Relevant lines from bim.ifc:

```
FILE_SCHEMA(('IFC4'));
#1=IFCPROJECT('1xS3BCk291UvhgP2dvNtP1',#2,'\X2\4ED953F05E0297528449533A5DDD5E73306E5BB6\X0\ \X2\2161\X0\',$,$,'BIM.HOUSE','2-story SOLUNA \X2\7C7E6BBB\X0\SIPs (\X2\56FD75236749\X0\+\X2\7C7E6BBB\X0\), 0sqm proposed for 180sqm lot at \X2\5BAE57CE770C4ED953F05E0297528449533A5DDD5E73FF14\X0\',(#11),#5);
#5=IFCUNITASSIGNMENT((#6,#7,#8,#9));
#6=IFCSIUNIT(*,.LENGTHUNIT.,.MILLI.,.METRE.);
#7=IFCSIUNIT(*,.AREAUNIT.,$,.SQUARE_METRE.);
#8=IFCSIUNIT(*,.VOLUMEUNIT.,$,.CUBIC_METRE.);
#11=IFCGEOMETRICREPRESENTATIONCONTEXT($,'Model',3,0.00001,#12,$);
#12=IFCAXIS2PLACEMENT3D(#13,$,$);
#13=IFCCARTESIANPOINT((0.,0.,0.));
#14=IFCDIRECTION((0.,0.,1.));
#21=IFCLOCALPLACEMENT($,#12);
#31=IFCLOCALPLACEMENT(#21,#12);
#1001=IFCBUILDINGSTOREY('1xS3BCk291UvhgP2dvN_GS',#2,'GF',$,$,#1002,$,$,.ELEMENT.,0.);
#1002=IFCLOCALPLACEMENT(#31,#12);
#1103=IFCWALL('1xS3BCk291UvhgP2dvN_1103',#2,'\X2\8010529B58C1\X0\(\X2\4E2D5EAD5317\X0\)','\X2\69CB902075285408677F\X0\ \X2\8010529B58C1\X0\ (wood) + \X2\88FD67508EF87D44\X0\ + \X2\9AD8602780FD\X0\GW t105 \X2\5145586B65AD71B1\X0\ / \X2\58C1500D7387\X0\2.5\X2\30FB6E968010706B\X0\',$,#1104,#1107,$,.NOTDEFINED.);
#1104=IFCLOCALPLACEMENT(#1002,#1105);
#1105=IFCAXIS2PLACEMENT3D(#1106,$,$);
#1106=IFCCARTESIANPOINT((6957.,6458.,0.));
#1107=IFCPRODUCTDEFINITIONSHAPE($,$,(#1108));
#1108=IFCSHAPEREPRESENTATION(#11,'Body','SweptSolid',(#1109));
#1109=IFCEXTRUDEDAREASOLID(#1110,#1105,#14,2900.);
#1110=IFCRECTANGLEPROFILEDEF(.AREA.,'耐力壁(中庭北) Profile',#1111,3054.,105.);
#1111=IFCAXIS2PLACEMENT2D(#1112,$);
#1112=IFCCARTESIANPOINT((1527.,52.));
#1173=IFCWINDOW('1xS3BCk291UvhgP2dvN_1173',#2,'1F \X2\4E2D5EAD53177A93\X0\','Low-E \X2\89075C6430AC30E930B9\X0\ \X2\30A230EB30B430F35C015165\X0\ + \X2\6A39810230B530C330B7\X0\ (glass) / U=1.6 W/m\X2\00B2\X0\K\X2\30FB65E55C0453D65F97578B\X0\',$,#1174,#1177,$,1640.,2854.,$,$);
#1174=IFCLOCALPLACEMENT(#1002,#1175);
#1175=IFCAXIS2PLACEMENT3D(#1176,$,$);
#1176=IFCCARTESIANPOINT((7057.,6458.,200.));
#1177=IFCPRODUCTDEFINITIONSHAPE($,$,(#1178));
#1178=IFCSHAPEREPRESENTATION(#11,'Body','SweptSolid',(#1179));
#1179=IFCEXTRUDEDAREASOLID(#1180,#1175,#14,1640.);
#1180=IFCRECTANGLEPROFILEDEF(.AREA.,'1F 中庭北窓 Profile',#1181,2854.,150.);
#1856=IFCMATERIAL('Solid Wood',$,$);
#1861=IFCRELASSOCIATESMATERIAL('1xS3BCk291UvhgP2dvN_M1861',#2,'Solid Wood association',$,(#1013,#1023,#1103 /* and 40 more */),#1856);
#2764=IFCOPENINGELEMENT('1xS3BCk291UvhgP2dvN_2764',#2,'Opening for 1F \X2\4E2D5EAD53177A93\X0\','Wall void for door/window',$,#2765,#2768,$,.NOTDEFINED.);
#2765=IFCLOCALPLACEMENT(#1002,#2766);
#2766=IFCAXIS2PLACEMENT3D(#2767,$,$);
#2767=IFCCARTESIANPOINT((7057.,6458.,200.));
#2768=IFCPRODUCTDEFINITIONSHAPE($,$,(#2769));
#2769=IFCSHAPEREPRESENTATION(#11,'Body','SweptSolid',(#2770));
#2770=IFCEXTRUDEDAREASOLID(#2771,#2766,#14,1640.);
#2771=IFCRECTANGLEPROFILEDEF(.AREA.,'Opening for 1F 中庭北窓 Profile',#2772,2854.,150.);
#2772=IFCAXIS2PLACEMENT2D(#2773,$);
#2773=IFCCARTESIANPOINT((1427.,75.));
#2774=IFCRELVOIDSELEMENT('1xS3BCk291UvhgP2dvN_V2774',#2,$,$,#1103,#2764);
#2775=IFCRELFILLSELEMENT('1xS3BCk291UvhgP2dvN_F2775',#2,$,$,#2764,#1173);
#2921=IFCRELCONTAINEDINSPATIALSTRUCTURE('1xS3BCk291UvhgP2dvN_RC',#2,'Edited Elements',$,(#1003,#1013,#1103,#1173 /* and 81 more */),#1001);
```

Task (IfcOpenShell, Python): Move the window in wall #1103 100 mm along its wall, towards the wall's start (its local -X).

```python
import ifcopenshell
import ifcopenshell.api.geometry
import ifcopenshell.util.placement
import ifcopenshell.util.unit

model = ifcopenshell.open("bim.ifc")
unit_scale = ifcopenshell.util.unit.calculate_unit_scale(model)

window = model.by_guid("1xS3BCk291UvhgP2dvN_1173")
opening = window.FillsVoids[0].RelatingOpeningElement
wall = opening.VoidsElements[0].RelatingBuildingElement

wall_matrix = ifcopenshell.util.placement.get_local_placement(wall.ObjectPlacement)
shift = wall_matrix[:3, 0] * -0.1 / unit_scale
before = ifcopenshell.util.placement.get_local_placement(window.ObjectPlacement)[:3, 3].copy()

# The window is not placed relative to its opening, so move both.
for product in (opening, window):
    matrix = ifcopenshell.util.placement.get_local_placement(product.ObjectPlacement)
    matrix[:3, 3] += shift
    ifcopenshell.api.geometry.edit_object_placement(model, product=product, matrix=matrix, is_si=False)

after = ifcopenshell.util.placement.get_local_placement(window.ObjectPlacement)[:3, 3]
print("window moved by", (after - before).round(3) + 0.0)

model.write("bim_v2.ifc")
```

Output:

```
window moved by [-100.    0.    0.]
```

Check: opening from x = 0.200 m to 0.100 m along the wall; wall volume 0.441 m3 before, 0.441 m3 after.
